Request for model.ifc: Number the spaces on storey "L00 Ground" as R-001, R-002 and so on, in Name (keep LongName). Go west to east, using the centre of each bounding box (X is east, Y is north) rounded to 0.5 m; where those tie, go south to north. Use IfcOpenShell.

First a look at what the model holds.

```python
import ifcopenshell
import ifcopenshell.util.element
import ifcopenshell.util.placement

model = ifcopenshell.open("model.ifc")
print(model.schema)
storey = next(s for s in model.by_type("IfcBuildingStorey") if s.Name == "L00 Ground")
spaces = [e for e in ifcopenshell.util.element.get_decomposition(storey) if e.is_a("IfcSpace")]
for e in sorted(spaces, key=lambda e: e.id()):
    origin = ifcopenshell.util.placement.get_local_placement(e.ObjectPlacement)[:3, 3]
    print(e.id(), e.Name, e.LongName, origin.round(2) + 0.0, sep=" | ")
```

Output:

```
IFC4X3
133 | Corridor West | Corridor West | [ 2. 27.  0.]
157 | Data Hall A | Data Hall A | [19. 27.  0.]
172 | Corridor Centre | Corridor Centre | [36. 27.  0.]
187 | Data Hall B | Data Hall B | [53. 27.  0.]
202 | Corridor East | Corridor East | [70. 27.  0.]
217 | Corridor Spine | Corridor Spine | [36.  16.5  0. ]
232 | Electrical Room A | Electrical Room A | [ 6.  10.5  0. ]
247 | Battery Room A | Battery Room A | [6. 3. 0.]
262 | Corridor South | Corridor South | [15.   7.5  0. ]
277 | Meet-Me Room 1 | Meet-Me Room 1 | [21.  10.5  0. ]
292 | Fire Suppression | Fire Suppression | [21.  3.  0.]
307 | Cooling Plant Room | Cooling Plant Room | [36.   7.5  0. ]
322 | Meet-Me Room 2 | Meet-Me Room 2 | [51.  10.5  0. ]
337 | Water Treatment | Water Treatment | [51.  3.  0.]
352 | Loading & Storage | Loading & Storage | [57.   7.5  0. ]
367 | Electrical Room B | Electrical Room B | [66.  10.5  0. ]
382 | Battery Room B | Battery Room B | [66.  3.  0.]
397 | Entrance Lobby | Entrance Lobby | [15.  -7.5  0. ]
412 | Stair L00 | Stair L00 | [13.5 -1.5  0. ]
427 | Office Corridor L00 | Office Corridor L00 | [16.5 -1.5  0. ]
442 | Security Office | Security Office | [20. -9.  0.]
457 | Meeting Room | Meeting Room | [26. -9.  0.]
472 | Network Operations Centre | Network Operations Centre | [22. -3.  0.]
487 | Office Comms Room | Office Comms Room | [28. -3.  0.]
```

```python
import ifcopenshell
import ifcopenshell.geom
import ifcopenshell.util.element
import ifcopenshell.util.shape

model = ifcopenshell.open("model.ifc")
settings = ifcopenshell.geom.settings()
settings.set("use-world-coords", True)


def centre(element):
    shape = ifcopenshell.geom.create_shape(settings, element)
    return ifcopenshell.util.shape.get_bbox_centroid(shape.geometry)


storey = next(s for s in model.by_type("IfcBuildingStorey") if s.Name == "L00 Ground")
spaces = [e for e in ifcopenshell.util.element.get_decomposition(storey) if e.is_a("IfcSpace")]

# Insertion points can sit at a corner or the storey origin, so sort by the geometry (in metres).
centres = {e: centre(e) for e in spaces}
spaces.sort(key=lambda e: (round(centres[e][0] / 0.5), centres[e][1]))

for i, e in enumerate(spaces, start=1):
    number = f"R-0{i:02d}"
    e.Name = number
    print(e.id(), number)

model.write("model-out.ifc")
```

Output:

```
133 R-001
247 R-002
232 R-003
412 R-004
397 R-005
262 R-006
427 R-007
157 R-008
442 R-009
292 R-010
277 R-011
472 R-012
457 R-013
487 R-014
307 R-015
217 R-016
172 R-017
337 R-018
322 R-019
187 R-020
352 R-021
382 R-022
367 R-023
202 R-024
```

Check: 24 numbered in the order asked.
